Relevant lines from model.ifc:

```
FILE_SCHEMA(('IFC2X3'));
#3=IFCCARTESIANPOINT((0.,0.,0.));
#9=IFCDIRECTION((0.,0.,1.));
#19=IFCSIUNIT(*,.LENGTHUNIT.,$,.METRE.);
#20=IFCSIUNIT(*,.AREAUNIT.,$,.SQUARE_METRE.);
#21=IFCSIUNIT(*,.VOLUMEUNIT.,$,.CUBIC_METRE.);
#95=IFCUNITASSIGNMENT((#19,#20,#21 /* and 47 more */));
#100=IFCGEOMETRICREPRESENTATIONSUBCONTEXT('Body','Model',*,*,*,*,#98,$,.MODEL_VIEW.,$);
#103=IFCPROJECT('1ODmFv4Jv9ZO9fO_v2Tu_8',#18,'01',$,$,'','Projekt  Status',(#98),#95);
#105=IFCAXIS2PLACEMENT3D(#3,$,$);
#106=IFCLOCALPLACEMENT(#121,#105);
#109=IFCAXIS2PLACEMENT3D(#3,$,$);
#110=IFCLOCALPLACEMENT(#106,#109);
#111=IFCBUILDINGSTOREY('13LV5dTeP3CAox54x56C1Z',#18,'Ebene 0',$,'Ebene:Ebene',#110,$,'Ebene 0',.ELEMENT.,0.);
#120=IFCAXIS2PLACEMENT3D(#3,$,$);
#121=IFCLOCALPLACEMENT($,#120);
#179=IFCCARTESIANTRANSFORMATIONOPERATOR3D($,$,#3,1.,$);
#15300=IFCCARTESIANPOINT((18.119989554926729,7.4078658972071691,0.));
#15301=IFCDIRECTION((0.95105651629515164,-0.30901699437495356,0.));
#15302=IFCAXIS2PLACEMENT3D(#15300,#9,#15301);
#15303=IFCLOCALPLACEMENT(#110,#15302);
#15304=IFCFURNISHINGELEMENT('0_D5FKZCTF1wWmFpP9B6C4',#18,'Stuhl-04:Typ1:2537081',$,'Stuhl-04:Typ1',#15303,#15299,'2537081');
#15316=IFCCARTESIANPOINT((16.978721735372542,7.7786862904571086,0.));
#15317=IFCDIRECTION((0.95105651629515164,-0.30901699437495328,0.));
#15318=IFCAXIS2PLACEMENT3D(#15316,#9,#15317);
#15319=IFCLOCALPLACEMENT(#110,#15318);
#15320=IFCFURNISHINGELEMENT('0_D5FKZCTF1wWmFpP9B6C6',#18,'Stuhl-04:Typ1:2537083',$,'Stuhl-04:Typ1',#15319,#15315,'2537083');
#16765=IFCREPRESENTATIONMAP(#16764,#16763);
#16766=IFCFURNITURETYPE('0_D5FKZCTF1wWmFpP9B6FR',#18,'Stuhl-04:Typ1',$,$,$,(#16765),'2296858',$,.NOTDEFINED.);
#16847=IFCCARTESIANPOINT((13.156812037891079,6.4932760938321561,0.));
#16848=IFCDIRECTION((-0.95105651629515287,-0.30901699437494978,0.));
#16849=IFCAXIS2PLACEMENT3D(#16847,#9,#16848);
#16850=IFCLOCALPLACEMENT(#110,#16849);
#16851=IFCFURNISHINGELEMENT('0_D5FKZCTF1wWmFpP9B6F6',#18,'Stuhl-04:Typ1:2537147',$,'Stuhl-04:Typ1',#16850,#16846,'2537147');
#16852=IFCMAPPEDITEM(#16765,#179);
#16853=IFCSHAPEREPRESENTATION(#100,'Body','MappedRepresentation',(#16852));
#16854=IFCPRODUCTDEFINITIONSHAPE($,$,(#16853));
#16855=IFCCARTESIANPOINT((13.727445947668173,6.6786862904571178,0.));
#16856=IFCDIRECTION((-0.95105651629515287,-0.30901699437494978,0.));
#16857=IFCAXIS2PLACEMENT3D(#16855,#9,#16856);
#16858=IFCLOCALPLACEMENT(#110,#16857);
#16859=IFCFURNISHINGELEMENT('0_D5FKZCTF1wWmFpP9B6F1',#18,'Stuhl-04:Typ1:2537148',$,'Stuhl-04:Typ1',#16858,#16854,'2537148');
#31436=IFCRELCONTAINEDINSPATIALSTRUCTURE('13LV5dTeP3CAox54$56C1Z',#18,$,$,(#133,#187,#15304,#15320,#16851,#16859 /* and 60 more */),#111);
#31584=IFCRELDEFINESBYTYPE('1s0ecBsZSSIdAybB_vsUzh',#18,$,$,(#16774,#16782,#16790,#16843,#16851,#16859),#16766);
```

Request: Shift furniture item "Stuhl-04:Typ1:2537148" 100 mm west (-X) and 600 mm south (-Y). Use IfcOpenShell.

```python
import ifcopenshell
import ifcopenshell.api.geometry
import ifcopenshell.util.placement

model = ifcopenshell.open("model.ifc")

item = model.by_guid("0_D5FKZCTF1wWmFpP9B6F1")
matrix = ifcopenshell.util.placement.get_local_placement(item.ObjectPlacement)
matrix[0, 3] -= 0.1
matrix[1, 3] -= 0.6
ifcopenshell.api.geometry.edit_object_placement(model, product=item, matrix=matrix, is_si=False)

print(ifcopenshell.util.placement.get_local_placement(item.ObjectPlacement).round(3) + 0.0)

model.write("model_v2.ifc")
```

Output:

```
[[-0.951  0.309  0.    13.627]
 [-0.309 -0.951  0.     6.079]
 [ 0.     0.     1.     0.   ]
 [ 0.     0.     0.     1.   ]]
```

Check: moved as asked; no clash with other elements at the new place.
